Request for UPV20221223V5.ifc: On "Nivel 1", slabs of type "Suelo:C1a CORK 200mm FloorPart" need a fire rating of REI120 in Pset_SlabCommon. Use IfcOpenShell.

First a look at what the model holds.

```python
import ifcopenshell
import ifcopenshell.util.element

model = ifcopenshell.open("UPV20221223V5.ifc")
print(model.schema)
storey = next(s for s in model.by_type("IfcBuildingStorey") if s.Name == "Nivel 1")
slabs = [e for e in ifcopenshell.util.element.get_decomposition(storey) if e.is_a("IfcSlab")]
seen = {}
for e in slabs:
    element_type = ifcopenshell.util.element.get_type(e)
    key = (element_type.Name if element_type != e and element_type else None, ifcopenshell.util.element.get_pset(e, "Pset_SlabCommon", "FireRating"))
    seen[key] = seen.get(key, 0) + 1
for (name, value), count in sorted(seen.items(), key=str):
    print(count, "x", name, "|", value)
```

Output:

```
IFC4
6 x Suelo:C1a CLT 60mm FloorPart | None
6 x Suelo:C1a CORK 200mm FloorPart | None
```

```python
import ifcopenshell
import ifcopenshell.api.pset
import ifcopenshell.util.element

model = ifcopenshell.open("UPV20221223V5.ifc")

storey = next(s for s in model.by_type("IfcBuildingStorey") if s.Name == "Nivel 1")
slabs = [e for e in ifcopenshell.util.element.get_decomposition(storey) if e.is_a("IfcSlab")]

count = 0
for e in slabs:
    element_type = ifcopenshell.util.element.get_type(e)
    if element_type in (None, e) or element_type.Name != "Suelo:C1a CORK 200mm FloorPart":
        continue
    # add_pset returns the element's existing set when there is one.
    pset = ifcopenshell.api.pset.add_pset(model, product=e, name="Pset_SlabCommon")
    ifcopenshell.api.pset.edit_pset(model, pset=pset, properties={"FireRating": "REI120"})
    count += 1

print(count, "slabs updated")

model.write("UPV20221223V5_updated.ifc")
```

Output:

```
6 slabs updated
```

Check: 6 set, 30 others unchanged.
